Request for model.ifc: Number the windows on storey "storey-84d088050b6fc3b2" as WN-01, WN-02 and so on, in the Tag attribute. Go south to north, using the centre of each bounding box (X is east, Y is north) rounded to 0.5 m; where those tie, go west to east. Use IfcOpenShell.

First a look at what the model holds.

```python
import ifcopenshell
import ifcopenshell.util.element
import ifcopenshell.util.placement

model = ifcopenshell.open("model.ifc")
print(model.schema)
storey = next(s for s in model.by_type("IfcBuildingStorey") if s.Name == "storey-84d088050b6fc3b2")
windows = [e for e in ifcopenshell.util.element.get_decomposition(storey) if e.is_a("IfcWindow")]
for e in sorted(windows, key=lambda e: e.id()):
    origin = ifcopenshell.util.placement.get_local_placement(e.ObjectPlacement)[:3, 3]
    print(e.id(), e.Tag, e.Name, origin.round(2) + 0.0, sep=" | ")
```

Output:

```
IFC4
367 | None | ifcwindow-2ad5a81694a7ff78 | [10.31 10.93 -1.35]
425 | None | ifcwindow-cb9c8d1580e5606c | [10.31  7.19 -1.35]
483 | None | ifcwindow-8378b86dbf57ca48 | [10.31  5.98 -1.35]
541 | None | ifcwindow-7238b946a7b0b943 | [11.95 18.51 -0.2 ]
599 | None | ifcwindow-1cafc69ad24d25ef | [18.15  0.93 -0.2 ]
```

```python
import ifcopenshell
import ifcopenshell.geom
import ifcopenshell.util.element
import ifcopenshell.util.shape

model = ifcopenshell.open("model.ifc")
settings = ifcopenshell.geom.settings()
settings.set("use-world-coords", True)


def centre(element):
    shape = ifcopenshell.geom.create_shape(settings, element)
    return ifcopenshell.util.shape.get_bbox_centroid(shape.geometry)


storey = next(s for s in model.by_type("IfcBuildingStorey") if s.Name == "storey-84d088050b6fc3b2")
windows = [e for e in ifcopenshell.util.element.get_decomposition(storey) if e.is_a("IfcWindow")]

# Insertion points can sit at a corner or the storey origin, so sort by the geometry (in metres).
centres = {e: centre(e) for e in windows}
windows.sort(key=lambda e: (round(centres[e][1] / 0.5), centres[e][0]))

for i, e in enumerate(windows, start=1):
    number = f"WN-{i:02d}"
    e.Tag = number
    print(e.id(), number)

model.write("model-out.ifc")
```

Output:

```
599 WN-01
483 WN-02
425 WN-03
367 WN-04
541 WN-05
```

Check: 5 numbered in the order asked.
